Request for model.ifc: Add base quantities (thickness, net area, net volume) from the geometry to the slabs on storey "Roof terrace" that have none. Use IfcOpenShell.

First a look at what the model holds.

```python
import ifcopenshell
import ifcopenshell.util.element
import ifcopenshell.util.unit

model = ifcopenshell.open("model.ifc")
print(model.schema)
for unit_type in ("LENGTHUNIT", "AREAUNIT", "VOLUMEUNIT"):
    print(unit_type, ifcopenshell.util.unit.calculate_unit_scale(model, unit_type))
storey = next(s for s in model.by_type("IfcBuildingStorey") if s.Name == "Roof terrace")
slabs = [e for e in ifcopenshell.util.element.get_decomposition(storey) if e.is_a("IfcSlab")]
for e in sorted(slabs, key=lambda e: e.id()):
    print(e.id(), e.is_a(), e.Name, list(ifcopenshell.util.element.get_psets(e, qtos_only=True)), sep=" | ")
```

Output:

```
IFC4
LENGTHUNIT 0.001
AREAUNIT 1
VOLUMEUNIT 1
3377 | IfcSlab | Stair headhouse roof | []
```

```python
import ifcopenshell
import ifcopenshell.api.pset
import ifcopenshell.geom
import ifcopenshell.util.element
import ifcopenshell.util.shape
import ifcopenshell.util.unit

model = ifcopenshell.open("model.ifc")
unit_scale = ifcopenshell.util.unit.calculate_unit_scale(model)
area_scale = ifcopenshell.util.unit.calculate_unit_scale(model, "AREAUNIT")
volume_scale = ifcopenshell.util.unit.calculate_unit_scale(model, "VOLUMEUNIT")
settings = ifcopenshell.geom.settings()

storey = next(s for s in model.by_type("IfcBuildingStorey") if s.Name == "Roof terrace")
slabs = [e for e in ifcopenshell.util.element.get_decomposition(storey) if e.is_a("IfcSlab")]

for e in sorted(slabs, key=lambda e: e.id()):
    if ifcopenshell.util.element.get_psets(e, qtos_only=True, should_inherit=False):
        continue
    # Geometry comes back in metres, in the element's own axes.
    shape = ifcopenshell.geom.create_shape(settings, e)
    values = {
        "Width": ifcopenshell.util.shape.get_z(shape.geometry) / unit_scale,
        "NetArea": ifcopenshell.util.shape.get_footprint_area(shape.geometry) / area_scale,
        "NetVolume": ifcopenshell.util.shape.get_volume(shape.geometry) / volume_scale,
    }
    qto = ifcopenshell.api.pset.add_qto(model, product=e, name="Qto_SlabBaseQuantities")
    ifcopenshell.api.pset.edit_qto(model, qto=qto, properties=values)
    print(e.id(), {k: round(v, 3) for k, v in values.items()})

model.write("model-out.ifc")
```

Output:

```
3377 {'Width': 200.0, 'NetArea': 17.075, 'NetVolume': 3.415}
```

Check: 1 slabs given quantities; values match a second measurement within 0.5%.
